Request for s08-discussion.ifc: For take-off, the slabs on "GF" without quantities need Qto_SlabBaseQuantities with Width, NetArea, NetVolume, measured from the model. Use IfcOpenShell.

First a look at what the model holds.

```python
import ifcopenshell
import ifcopenshell.util.element
import ifcopenshell.util.unit

model = ifcopenshell.open("s08-discussion.ifc")
print(model.schema)
for unit_type in ("LENGTHUNIT", "AREAUNIT", "VOLUMEUNIT"):
    print(unit_type, ifcopenshell.util.unit.calculate_unit_scale(model, unit_type))
storey = next(s for s in model.by_type("IfcBuildingStorey") if s.Name == "GF")
slabs = [e for e in ifcopenshell.util.element.get_decomposition(storey) if e.is_a("IfcSlab")]
for e in sorted(slabs, key=lambda e: e.id()):
    print(e.id(), e.is_a(), e.Name, list(ifcopenshell.util.element.get_psets(e, qtos_only=True)), sep=" | ")
```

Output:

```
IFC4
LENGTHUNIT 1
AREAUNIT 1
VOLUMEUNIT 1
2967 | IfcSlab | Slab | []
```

```python
import ifcopenshell
import ifcopenshell.api.pset
import ifcopenshell.geom
import ifcopenshell.util.element
import ifcopenshell.util.shape
import ifcopenshell.util.unit

model = ifcopenshell.open("s08-discussion.ifc")
unit_scale = ifcopenshell.util.unit.calculate_unit_scale(model)
area_scale = ifcopenshell.util.unit.calculate_unit_scale(model, "AREAUNIT")
volume_scale = ifcopenshell.util.unit.calculate_unit_scale(model, "VOLUMEUNIT")
settings = ifcopenshell.geom.settings()

storey = next(s for s in model.by_type("IfcBuildingStorey") if s.Name == "GF")
slabs = [e for e in ifcopenshell.util.element.get_decomposition(storey) if e.is_a("IfcSlab")]

for e in sorted(slabs, key=lambda e: e.id()):
    if ifcopenshell.util.element.get_psets(e, qtos_only=True, should_inherit=False):
        continue
    # Geometry comes back in metres, in the element's own axes.
    shape = ifcopenshell.geom.create_shape(settings, e)
    values = {
        "Width": ifcopenshell.util.shape.get_z(shape.geometry) / unit_scale,
        "NetArea": ifcopenshell.util.shape.get_footprint_area(shape.geometry) / area_scale,
        "NetVolume": ifcopenshell.util.shape.get_volume(shape.geometry) / volume_scale,
    }
    qto = ifcopenshell.api.pset.add_qto(model, product=e, name="Qto_SlabBaseQuantities")
    ifcopenshell.api.pset.edit_qto(model, qto=qto, properties=values)
    print(e.id(), {k: round(v, 3) for k, v in values.items()})

model.write("s08-discussion-out.ifc")
```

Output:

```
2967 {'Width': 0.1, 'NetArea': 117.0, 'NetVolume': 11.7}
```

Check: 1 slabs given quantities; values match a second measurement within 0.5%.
